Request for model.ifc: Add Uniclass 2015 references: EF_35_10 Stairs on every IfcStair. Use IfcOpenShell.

First a look at what the model holds.

```python
import ifcopenshell

model = ifcopenshell.open("model.ifc")
print(model.schema)
print("classifications:", [c.Name for c in model.by_type("IfcClassification")])
for ifc_class in ("IfcDoor", "IfcRoof", "IfcStair", "IfcWall", "IfcWindow"):
    print(ifc_class, len(model.by_type(ifc_class)))
```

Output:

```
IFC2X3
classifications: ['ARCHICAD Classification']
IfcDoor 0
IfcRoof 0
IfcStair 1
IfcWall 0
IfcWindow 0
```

```python
import ifcopenshell
import ifcopenshell.api.classification

model = ifcopenshell.open("model.ifc")

# IFC2X3 requires Source and Edition and has no link from the project to the system.
system = model.create_entity("IfcClassification", Source="NBS", Edition="2015", Name="Uniclass 2015")

codes = {
    "IfcStair": ("EF_35_10", "Stairs"),
}
for ifc_class, (code, name) in codes.items():
    products = model.by_type(ifc_class)
    ifcopenshell.api.classification.add_reference(
        model, products=products, classification=system, identification=code, name=name
    )
    print(code, len(products))

model.write("model_updated.ifc")
```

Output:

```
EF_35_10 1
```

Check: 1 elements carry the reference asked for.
